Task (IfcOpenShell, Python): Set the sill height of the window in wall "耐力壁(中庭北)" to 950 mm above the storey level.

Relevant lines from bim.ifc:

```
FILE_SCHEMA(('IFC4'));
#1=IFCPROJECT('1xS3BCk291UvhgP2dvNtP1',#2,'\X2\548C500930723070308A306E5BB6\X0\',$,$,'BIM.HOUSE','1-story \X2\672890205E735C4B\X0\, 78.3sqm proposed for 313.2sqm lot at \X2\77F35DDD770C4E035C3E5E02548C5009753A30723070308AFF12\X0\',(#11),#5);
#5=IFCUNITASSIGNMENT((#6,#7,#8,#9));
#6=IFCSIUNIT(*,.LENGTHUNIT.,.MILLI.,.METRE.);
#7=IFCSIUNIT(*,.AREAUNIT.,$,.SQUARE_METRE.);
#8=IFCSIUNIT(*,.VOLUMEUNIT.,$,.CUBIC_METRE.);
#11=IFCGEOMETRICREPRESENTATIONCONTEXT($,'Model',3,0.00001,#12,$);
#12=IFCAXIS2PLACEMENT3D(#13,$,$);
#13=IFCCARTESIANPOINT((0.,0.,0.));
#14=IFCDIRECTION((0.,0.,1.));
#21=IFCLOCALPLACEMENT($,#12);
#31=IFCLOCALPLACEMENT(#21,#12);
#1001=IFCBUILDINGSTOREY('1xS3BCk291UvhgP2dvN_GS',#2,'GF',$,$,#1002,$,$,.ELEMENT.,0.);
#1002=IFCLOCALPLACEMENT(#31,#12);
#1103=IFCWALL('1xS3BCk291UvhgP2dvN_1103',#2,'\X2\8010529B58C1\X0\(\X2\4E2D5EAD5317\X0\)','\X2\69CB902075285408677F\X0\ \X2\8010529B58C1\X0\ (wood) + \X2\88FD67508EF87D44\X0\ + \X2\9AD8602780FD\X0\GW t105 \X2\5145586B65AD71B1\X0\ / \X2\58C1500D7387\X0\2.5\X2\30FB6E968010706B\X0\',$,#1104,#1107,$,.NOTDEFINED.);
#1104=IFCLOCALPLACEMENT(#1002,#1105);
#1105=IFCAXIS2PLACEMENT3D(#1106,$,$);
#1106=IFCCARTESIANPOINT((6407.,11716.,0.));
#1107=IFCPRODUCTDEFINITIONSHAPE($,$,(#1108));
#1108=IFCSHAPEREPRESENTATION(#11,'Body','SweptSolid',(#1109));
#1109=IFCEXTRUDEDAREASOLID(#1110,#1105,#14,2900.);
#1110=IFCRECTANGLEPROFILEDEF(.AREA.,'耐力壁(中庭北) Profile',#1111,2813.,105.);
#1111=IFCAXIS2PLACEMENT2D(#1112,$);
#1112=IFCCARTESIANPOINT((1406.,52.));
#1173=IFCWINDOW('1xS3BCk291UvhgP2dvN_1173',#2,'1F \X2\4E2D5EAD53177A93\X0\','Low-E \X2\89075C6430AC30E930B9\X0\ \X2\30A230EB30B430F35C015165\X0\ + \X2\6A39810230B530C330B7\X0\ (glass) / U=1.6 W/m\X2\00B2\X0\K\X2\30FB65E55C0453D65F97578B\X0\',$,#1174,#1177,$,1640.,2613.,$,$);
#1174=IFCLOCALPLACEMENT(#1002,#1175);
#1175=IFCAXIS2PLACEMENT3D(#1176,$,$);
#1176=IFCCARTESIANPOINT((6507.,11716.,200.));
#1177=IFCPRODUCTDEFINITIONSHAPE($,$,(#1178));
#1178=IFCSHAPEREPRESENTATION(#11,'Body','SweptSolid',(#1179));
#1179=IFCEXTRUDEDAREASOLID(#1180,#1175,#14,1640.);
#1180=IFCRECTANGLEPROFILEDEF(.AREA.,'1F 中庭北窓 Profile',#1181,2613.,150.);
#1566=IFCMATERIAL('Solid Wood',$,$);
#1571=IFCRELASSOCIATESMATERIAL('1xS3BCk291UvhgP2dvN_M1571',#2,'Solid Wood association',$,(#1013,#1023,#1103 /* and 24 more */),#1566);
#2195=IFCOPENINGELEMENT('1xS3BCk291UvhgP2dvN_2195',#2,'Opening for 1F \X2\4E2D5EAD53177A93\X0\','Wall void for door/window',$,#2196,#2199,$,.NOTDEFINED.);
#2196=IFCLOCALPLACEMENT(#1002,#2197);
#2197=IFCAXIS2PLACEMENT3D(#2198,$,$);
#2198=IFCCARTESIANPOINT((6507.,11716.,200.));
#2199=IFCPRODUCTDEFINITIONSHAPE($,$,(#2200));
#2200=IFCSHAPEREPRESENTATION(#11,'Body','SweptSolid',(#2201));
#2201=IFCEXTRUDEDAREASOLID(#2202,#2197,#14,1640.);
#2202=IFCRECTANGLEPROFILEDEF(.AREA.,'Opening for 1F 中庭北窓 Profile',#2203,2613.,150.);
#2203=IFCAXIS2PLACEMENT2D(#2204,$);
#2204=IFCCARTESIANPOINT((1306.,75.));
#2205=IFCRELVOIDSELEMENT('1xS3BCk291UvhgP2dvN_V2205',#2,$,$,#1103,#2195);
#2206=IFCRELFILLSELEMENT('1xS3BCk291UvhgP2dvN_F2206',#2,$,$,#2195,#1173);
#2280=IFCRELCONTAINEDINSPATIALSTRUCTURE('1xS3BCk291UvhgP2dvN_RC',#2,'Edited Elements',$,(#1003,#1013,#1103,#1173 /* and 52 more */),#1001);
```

```python
import numpy as np
import ifcopenshell
import ifcopenshell.api.geometry
import ifcopenshell.geom
import ifcopenshell.util.element
import ifcopenshell.util.placement
import ifcopenshell.util.shape
import ifcopenshell.util.unit

model = ifcopenshell.open("bim.ifc")
unit_scale = ifcopenshell.util.unit.calculate_unit_scale(model)

window = model.by_guid("1xS3BCk291UvhgP2dvN_1173")
opening = window.FillsVoids[0].RelatingOpeningElement
storey = ifcopenshell.util.element.get_container(window, ifc_class="IfcBuildingStorey")
level = ifcopenshell.util.placement.get_local_placement(storey.ObjectPlacement)[2, 3]

# The opening's origin need not be at the sill, so measure its lowest point.
shape = ifcopenshell.geom.create_shape(ifcopenshell.geom.settings(), opening)
bottom = ifcopenshell.util.shape.get_shape_bottom_elevation(shape, shape.geometry) / unit_scale
dz = level + 950.0 - bottom

shift = np.array([0.0, 0.0, dz])
# The window is not placed relative to its opening, so move both.
for product in (opening, window):
    matrix = ifcopenshell.util.placement.get_local_placement(product.ObjectPlacement)
    matrix[:3, 3] += shift
    ifcopenshell.api.geometry.edit_object_placement(model, product=product, matrix=matrix, is_si=False)

print(f"moved by {dz * unit_scale:+.3f} m")

model.write("bim_updated.ifc")
```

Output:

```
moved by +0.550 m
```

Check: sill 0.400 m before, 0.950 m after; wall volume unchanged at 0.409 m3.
